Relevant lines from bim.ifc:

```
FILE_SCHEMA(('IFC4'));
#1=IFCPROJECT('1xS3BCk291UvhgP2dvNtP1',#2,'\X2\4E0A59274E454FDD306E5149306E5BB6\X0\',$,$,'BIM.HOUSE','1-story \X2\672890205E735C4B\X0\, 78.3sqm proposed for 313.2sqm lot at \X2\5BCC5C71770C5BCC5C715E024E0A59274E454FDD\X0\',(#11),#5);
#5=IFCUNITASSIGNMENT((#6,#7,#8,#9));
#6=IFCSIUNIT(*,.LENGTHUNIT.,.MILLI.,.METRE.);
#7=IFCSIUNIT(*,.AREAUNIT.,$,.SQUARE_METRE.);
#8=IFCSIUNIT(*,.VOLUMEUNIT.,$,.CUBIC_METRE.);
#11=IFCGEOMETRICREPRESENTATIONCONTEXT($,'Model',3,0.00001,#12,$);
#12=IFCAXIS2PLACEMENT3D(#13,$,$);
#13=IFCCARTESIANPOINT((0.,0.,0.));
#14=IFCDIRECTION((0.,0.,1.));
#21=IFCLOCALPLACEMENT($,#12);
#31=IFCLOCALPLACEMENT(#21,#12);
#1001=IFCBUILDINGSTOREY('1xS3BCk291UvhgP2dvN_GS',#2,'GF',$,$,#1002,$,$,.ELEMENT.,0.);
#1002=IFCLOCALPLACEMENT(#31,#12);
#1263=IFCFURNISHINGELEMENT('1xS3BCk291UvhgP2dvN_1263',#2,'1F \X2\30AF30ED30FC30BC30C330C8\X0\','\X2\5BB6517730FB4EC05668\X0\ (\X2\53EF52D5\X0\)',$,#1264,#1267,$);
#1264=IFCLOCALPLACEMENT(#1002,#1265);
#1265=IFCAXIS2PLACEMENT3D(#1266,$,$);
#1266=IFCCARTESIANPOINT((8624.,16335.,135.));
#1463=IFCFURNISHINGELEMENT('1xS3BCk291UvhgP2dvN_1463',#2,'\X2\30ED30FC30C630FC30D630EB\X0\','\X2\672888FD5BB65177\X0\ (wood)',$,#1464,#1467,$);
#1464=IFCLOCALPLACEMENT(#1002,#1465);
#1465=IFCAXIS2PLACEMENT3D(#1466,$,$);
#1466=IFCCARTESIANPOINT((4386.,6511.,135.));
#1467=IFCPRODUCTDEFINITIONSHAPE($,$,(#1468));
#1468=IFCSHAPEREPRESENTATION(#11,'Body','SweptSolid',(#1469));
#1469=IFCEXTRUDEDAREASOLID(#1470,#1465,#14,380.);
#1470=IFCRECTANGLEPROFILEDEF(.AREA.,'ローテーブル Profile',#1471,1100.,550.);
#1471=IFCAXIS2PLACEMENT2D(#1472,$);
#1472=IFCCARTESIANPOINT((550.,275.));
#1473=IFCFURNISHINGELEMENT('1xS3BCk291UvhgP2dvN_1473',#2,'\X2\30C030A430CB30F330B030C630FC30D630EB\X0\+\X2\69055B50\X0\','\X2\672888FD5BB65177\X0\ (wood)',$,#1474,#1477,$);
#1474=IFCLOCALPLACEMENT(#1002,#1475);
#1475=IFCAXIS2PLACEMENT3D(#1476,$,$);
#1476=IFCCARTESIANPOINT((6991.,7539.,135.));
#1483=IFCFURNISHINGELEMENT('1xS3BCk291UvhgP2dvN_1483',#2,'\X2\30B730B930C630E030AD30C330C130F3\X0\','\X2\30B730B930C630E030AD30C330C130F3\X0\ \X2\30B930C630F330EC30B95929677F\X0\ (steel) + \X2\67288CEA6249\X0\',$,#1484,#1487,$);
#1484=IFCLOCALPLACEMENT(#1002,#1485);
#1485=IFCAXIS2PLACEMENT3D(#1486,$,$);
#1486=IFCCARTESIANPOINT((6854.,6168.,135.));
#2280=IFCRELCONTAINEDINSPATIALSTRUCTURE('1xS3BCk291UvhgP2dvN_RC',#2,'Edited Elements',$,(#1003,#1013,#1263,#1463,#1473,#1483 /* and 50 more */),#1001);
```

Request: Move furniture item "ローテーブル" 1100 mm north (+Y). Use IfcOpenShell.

```python
import ifcopenshell
import ifcopenshell.api.geometry
import ifcopenshell.util.placement
import ifcopenshell.util.unit

model = ifcopenshell.open("bim.ifc")
unit_scale = ifcopenshell.util.unit.calculate_unit_scale(model)

item = model.by_id(1463)
matrix = ifcopenshell.util.placement.get_local_placement(item.ObjectPlacement)
matrix[1, 3] += 1.1 / unit_scale
ifcopenshell.api.geometry.edit_object_placement(model, product=item, matrix=matrix, is_si=False)

print(ifcopenshell.util.placement.get_local_placement(item.ObjectPlacement).round(3) + 0.0)

model.write("bim_updated.ifc")
```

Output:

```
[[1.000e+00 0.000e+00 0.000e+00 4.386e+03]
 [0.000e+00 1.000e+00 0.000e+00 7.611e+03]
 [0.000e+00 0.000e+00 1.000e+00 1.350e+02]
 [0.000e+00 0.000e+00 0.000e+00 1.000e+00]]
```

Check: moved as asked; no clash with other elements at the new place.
